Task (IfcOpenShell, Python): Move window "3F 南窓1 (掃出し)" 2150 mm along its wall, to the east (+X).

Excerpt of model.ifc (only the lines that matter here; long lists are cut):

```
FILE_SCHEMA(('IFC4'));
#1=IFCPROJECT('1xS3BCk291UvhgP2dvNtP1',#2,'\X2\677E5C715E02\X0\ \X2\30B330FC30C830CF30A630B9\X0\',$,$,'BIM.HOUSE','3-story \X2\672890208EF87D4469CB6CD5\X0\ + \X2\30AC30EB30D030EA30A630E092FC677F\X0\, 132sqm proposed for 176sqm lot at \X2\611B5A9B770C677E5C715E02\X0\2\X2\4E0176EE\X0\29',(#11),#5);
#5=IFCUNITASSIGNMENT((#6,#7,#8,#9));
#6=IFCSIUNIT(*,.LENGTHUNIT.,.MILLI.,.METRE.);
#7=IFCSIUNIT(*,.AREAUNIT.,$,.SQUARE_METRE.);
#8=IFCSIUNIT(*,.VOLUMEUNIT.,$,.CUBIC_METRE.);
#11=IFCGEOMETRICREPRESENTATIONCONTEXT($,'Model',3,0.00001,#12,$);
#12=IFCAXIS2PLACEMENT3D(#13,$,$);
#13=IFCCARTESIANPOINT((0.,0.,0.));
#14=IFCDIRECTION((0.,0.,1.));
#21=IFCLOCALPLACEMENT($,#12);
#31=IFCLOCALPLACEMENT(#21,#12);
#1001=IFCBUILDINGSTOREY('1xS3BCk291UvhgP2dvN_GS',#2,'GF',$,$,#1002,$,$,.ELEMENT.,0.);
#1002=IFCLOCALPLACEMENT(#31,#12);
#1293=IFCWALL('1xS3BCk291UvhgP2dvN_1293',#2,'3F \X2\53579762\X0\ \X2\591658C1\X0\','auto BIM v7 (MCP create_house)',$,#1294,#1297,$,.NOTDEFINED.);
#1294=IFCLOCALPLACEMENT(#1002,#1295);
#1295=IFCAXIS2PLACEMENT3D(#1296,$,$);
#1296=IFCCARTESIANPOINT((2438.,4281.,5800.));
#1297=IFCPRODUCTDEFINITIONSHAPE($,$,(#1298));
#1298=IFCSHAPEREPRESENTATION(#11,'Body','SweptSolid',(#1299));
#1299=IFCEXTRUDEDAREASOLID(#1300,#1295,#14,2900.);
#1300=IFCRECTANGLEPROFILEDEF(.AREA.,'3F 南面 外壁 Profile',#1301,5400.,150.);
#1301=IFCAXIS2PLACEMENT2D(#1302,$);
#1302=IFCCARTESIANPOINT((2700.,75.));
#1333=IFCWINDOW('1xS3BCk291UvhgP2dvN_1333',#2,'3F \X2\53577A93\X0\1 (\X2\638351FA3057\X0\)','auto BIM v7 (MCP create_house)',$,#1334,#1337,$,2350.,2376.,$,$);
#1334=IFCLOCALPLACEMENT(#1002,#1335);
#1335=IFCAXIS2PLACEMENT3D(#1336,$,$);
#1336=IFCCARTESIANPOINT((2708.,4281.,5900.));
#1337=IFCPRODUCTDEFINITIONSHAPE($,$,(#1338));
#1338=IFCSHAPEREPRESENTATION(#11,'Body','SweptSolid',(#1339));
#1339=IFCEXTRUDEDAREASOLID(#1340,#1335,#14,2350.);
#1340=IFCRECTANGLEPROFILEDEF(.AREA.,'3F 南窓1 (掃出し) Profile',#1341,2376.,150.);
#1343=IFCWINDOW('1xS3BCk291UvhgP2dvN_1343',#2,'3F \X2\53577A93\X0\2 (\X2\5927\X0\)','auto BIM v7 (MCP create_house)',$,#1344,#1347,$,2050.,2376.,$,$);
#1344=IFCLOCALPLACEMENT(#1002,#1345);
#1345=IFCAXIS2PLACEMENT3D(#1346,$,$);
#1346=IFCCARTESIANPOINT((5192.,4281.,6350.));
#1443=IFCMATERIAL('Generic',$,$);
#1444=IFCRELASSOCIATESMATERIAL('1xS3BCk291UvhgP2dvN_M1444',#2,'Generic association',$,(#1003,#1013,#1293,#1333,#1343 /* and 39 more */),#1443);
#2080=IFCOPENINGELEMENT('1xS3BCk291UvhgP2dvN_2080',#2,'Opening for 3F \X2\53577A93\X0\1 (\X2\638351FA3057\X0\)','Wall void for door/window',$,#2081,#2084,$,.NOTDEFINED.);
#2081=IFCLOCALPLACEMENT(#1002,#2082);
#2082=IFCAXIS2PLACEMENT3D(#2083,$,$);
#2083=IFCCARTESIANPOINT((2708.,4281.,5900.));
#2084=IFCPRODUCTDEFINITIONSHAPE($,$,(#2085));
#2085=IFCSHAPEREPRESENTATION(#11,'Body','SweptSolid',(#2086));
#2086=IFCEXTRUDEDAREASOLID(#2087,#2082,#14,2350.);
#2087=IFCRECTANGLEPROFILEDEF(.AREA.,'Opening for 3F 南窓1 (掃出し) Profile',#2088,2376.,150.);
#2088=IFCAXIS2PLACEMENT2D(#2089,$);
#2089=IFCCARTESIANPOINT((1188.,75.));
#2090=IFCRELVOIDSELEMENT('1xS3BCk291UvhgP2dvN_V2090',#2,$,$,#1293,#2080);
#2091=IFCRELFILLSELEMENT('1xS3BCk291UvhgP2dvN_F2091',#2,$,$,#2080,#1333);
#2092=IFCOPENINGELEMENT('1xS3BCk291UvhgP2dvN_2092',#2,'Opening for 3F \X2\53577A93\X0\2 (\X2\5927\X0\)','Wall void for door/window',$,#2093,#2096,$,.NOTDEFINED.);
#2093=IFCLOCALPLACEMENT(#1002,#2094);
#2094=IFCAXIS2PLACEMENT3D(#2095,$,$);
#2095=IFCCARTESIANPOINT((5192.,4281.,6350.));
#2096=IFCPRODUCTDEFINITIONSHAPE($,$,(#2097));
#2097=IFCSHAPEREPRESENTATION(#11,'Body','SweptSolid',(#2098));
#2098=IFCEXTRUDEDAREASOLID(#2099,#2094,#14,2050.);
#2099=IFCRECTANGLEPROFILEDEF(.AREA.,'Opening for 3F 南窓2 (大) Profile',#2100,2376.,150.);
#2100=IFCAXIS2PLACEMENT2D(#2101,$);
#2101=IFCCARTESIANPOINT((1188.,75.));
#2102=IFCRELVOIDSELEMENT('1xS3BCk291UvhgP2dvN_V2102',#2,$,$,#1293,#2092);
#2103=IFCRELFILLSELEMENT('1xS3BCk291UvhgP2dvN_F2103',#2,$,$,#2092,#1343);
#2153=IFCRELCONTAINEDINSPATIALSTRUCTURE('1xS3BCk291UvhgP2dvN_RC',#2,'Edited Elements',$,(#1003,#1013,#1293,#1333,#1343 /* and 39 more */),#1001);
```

```python
import ifcopenshell
import ifcopenshell.api.geometry
import ifcopenshell.util.placement

model = ifcopenshell.open("model.ifc")

window = model.by_guid("1xS3BCk291UvhgP2dvN_1333")
opening = window.FillsVoids[0].RelatingOpeningElement
wall = opening.VoidsElements[0].RelatingBuildingElement

wall_matrix = ifcopenshell.util.placement.get_local_placement(wall.ObjectPlacement)
shift = wall_matrix[:3, 0] * 2150.0
before = ifcopenshell.util.placement.get_local_placement(window.ObjectPlacement)[:3, 3].copy()

# The window is not placed relative to its opening, so move both.
for product in (opening, window):
    matrix = ifcopenshell.util.placement.get_local_placement(product.ObjectPlacement)
    matrix[:3, 3] += shift
    ifcopenshell.api.geometry.edit_object_placement(model, product=product, matrix=matrix, is_si=False)

after = ifcopenshell.util.placement.get_local_placement(window.ObjectPlacement)[:3, 3]
print("window moved by", (after - before).round(3) + 0.0)

model.write("model_edited.ifc")
```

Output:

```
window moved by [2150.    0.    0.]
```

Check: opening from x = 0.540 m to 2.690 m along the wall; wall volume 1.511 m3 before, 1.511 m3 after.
